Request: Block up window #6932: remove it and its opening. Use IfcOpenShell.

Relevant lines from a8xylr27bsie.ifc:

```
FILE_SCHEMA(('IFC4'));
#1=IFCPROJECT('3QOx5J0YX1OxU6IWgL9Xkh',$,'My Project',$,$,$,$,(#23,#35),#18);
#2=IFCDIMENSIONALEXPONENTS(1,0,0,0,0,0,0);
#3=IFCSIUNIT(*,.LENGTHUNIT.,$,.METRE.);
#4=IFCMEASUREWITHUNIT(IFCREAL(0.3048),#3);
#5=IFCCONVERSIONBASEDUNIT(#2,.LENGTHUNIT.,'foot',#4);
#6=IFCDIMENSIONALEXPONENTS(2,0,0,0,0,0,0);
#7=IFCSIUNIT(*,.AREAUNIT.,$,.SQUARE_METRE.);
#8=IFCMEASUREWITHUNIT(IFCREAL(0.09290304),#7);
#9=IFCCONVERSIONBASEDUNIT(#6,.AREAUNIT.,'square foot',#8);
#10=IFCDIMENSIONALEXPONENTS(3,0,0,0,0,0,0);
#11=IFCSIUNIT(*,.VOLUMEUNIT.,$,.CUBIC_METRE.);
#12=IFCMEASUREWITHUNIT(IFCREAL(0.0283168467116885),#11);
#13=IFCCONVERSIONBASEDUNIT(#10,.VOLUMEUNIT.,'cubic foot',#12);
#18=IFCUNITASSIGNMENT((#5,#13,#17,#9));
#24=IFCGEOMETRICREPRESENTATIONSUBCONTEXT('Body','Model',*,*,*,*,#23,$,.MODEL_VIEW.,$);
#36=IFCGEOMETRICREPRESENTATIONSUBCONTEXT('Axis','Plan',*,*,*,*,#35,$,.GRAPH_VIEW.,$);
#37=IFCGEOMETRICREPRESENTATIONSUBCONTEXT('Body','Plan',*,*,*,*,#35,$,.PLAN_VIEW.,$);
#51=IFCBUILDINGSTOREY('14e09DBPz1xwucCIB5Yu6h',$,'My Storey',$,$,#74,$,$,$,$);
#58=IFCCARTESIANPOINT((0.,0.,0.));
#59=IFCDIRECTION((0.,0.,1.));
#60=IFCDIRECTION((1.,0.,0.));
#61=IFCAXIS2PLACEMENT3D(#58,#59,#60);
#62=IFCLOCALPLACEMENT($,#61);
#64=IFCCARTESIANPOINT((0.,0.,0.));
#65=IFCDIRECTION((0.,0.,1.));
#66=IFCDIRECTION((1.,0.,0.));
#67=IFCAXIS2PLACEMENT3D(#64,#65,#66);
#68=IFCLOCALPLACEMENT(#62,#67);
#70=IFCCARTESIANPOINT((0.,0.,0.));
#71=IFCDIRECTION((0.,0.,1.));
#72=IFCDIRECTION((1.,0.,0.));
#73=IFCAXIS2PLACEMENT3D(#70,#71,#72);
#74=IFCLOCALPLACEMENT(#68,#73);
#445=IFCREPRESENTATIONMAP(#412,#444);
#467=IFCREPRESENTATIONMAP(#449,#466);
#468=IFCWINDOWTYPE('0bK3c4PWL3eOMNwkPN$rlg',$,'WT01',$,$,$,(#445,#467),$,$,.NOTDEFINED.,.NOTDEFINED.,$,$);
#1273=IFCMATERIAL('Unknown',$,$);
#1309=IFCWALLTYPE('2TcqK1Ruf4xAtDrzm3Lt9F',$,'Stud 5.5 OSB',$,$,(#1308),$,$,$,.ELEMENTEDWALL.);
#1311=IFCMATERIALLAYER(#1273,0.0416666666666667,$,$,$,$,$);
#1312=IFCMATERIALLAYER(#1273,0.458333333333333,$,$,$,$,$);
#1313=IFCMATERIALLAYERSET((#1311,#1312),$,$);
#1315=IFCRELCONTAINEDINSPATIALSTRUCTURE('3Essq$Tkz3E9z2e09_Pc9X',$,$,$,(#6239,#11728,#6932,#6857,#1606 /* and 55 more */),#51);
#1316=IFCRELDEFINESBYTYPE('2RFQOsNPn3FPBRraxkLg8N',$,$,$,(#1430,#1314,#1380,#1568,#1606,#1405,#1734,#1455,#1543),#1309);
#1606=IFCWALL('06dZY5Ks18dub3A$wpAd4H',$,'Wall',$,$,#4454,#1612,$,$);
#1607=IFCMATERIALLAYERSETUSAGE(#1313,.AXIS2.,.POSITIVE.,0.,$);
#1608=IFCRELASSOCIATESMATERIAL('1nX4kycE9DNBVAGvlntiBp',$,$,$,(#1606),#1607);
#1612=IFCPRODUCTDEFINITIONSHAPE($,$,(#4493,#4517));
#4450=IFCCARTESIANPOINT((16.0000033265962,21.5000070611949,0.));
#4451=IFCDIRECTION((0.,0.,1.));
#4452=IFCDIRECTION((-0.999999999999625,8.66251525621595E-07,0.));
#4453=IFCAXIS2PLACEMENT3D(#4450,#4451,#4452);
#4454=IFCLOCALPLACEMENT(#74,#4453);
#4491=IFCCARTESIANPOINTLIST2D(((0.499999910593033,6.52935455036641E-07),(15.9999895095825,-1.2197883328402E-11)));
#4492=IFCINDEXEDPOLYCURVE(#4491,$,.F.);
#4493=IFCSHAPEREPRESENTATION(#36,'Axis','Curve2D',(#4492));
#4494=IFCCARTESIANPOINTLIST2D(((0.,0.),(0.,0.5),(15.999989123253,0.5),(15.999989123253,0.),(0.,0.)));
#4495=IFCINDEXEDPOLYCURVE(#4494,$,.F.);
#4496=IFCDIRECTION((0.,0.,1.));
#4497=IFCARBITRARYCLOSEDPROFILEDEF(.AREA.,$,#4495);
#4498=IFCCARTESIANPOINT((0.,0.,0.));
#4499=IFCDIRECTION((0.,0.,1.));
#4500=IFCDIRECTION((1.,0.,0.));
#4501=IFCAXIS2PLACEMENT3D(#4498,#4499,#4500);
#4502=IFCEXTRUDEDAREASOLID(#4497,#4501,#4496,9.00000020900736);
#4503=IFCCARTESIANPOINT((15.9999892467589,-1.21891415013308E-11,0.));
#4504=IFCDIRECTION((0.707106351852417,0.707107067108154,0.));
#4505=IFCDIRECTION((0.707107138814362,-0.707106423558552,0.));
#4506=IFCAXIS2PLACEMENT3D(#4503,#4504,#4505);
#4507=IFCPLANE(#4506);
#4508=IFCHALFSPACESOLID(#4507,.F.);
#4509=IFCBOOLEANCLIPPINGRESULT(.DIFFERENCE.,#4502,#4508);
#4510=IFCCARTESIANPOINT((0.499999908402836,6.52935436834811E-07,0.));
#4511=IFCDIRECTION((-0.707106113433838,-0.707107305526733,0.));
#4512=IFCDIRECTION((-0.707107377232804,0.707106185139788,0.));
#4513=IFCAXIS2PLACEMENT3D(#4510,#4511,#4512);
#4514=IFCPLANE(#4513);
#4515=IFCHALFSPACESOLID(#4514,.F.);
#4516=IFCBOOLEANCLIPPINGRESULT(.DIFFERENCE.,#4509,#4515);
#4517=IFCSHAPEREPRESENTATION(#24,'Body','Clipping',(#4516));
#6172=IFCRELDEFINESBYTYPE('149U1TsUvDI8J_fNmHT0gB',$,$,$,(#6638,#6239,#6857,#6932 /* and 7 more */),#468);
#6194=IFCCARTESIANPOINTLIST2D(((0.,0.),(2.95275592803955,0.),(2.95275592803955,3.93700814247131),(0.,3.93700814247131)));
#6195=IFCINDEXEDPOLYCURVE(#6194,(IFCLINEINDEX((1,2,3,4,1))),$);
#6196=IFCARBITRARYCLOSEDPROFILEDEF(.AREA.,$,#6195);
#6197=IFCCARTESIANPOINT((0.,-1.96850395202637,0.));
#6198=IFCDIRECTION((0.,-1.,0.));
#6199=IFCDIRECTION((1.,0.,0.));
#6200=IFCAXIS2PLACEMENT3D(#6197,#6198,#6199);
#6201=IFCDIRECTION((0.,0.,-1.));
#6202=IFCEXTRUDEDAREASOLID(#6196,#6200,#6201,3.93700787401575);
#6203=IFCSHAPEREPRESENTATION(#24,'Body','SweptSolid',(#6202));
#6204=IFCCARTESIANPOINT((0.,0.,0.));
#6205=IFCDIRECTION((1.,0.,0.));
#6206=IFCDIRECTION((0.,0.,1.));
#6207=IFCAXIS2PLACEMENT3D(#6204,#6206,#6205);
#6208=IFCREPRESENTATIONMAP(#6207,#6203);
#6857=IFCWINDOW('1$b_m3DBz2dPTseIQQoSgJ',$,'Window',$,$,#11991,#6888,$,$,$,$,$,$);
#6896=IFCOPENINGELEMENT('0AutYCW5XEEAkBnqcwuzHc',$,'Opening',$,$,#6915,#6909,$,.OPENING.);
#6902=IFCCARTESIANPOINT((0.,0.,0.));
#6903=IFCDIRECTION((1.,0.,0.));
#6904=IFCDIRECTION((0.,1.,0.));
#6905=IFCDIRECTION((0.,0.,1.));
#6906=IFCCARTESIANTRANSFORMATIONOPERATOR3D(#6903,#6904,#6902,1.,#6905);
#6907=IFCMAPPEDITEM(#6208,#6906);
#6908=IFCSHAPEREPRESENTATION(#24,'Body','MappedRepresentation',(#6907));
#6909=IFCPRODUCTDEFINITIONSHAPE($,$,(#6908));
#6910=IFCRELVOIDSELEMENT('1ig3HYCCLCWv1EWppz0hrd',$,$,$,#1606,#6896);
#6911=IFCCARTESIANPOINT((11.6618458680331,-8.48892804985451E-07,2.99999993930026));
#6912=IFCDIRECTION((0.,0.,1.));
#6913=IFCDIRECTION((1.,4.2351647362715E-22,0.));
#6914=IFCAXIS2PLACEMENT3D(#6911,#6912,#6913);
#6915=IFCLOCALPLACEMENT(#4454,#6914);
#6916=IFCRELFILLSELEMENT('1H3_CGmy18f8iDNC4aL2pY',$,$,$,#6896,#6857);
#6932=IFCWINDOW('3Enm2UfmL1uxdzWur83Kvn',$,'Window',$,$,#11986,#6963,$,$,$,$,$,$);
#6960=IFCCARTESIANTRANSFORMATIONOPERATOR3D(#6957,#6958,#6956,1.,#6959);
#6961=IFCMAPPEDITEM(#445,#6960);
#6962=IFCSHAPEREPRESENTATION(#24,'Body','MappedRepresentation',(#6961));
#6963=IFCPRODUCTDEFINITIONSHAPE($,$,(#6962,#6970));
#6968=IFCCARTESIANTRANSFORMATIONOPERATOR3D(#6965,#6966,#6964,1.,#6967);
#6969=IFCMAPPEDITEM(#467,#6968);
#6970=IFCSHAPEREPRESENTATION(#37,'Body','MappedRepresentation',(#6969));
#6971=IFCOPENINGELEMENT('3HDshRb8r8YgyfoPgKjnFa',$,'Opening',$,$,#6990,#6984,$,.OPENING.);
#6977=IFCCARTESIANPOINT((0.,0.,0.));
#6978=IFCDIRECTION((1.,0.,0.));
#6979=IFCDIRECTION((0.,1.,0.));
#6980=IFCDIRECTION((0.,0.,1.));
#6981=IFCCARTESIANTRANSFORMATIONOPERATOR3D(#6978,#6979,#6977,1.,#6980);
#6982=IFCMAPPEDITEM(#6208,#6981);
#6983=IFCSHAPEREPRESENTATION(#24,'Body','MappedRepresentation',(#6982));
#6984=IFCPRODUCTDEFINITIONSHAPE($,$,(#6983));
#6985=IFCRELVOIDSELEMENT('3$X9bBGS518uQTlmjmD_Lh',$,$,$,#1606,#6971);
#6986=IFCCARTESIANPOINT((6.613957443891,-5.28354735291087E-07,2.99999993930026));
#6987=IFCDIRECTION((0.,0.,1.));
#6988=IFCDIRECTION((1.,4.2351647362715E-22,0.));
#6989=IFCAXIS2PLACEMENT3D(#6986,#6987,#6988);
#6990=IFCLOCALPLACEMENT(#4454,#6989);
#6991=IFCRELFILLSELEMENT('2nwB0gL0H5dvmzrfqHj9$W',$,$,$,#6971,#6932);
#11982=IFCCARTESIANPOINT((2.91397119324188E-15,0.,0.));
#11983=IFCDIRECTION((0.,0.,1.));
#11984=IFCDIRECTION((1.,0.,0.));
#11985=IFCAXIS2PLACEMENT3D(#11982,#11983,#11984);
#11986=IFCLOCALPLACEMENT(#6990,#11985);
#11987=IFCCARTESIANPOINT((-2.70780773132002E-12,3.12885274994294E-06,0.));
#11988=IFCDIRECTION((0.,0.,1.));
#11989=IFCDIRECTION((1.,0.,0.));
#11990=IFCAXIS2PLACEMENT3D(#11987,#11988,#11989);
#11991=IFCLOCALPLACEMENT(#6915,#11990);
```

```python
import ifcopenshell
import ifcopenshell.api.feature
import ifcopenshell.api.root
import ifcopenshell.geom
import ifcopenshell.util.shape

model = ifcopenshell.open("a8xylr27bsie.ifc")
settings = ifcopenshell.geom.settings()


def volume(element):
    """Net volume in cubic metres, openings subtracted."""
    shape = ifcopenshell.geom.create_shape(settings, element)
    return ifcopenshell.util.shape.get_volume(shape.geometry)


window = model.by_id(6932)
opening = window.FillsVoids[0].RelatingOpeningElement
wall = opening.VoidsElements[0].RelatingBuildingElement
before = volume(wall)

ifcopenshell.api.root.remove_product(model, product=window)
ifcopenshell.api.feature.remove_feature(model, feature=opening)

after = volume(wall)

print(f"wall volume {before:.3f} -> {after:.3f} m3")

model.write("a8xylr27bsie_edited.ifc")
```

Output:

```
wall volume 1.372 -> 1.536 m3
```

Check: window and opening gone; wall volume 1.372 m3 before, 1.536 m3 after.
